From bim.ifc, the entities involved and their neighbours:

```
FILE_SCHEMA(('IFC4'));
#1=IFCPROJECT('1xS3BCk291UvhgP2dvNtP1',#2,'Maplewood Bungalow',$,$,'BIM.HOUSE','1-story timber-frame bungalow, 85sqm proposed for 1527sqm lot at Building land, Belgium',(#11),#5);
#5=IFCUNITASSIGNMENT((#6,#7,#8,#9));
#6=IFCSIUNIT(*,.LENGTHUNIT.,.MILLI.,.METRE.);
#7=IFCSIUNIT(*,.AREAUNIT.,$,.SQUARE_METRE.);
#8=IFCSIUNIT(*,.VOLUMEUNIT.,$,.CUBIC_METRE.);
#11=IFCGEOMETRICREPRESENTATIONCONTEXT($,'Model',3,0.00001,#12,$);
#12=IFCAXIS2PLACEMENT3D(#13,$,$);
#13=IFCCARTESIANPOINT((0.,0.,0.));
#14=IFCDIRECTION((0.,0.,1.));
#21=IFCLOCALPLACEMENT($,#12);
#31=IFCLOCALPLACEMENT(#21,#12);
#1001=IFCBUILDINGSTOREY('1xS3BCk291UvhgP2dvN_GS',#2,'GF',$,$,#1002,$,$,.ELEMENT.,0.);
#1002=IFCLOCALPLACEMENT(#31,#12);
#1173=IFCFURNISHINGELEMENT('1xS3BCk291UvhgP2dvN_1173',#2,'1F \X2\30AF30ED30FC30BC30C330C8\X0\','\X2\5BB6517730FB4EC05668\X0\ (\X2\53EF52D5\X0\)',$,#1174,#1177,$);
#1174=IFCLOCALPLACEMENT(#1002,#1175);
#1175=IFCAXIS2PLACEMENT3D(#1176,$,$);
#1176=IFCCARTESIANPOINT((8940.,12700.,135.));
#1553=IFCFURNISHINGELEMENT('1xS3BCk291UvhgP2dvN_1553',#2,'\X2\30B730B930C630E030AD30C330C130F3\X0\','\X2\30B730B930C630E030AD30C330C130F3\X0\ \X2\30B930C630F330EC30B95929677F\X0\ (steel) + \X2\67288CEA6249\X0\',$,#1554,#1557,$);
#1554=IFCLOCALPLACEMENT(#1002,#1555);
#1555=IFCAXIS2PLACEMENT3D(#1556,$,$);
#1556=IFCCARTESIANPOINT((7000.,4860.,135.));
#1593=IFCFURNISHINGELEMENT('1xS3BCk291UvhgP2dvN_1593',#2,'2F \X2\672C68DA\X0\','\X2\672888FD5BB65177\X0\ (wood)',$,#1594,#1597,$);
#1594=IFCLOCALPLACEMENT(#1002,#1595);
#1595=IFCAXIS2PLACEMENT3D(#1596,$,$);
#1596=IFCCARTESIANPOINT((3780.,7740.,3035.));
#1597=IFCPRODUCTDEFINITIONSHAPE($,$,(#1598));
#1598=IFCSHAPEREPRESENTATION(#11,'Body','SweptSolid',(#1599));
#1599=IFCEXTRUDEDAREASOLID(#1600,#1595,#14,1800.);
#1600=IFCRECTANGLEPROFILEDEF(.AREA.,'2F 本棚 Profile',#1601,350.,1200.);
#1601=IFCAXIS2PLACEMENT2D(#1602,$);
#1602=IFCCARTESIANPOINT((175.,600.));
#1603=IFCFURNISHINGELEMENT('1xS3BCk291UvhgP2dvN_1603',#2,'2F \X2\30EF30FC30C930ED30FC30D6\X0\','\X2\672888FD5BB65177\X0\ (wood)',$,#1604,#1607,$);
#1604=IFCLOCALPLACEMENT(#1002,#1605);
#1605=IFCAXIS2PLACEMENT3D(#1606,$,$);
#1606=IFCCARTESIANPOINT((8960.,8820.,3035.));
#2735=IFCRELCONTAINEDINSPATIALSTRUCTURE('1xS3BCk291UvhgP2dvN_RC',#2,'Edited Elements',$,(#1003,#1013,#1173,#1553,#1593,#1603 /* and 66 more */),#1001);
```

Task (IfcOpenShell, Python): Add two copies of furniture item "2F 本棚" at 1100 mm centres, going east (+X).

```python
import numpy as np
import ifcopenshell
import ifcopenshell.api.geometry
import ifcopenshell.api.root
import ifcopenshell.util.element
import ifcopenshell.util.placement
import ifcopenshell.util.unit

model = ifcopenshell.open("bim.ifc")
unit_scale = ifcopenshell.util.unit.calculate_unit_scale(model)


def reuse_history(source, copy):
    """copy_class also copies each property set's owner history, people and application; keep the originals."""
    for rel in copy.IsDefinedBy:
        if rel.is_a("IfcRelDefinesByProperties") and (history := rel.RelatingPropertyDefinition.OwnerHistory):
            rel.RelatingPropertyDefinition.OwnerHistory = source.OwnerHistory
            ifcopenshell.util.element.remove_deep2(model, history)


source = model.by_guid("1xS3BCk291UvhgP2dvN_1593")
base = ifcopenshell.util.placement.get_local_placement(source.ObjectPlacement)
step = np.array([1.0, 0.0, 0.0]) * 1.1 / unit_scale

for i in range(1, 3):
    copy = ifcopenshell.api.root.copy_class(model, product=source)
    copy.Representation = ifcopenshell.util.element.copy_deep(
        model, source.Representation, exclude=["IfcGeometricRepresentationContext", "IfcRepresentationMap"]
    )
    reuse_history(source, copy)
    matrix = base.copy()
    matrix[:3, 3] += i * step
    print("added at", matrix[:3, 3].round(3) + 0.0)
    ifcopenshell.api.geometry.edit_object_placement(model, product=copy, matrix=matrix, is_si=False)

model.write("bim_rev.ifc")
```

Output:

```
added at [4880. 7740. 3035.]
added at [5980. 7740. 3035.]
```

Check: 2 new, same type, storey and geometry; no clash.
